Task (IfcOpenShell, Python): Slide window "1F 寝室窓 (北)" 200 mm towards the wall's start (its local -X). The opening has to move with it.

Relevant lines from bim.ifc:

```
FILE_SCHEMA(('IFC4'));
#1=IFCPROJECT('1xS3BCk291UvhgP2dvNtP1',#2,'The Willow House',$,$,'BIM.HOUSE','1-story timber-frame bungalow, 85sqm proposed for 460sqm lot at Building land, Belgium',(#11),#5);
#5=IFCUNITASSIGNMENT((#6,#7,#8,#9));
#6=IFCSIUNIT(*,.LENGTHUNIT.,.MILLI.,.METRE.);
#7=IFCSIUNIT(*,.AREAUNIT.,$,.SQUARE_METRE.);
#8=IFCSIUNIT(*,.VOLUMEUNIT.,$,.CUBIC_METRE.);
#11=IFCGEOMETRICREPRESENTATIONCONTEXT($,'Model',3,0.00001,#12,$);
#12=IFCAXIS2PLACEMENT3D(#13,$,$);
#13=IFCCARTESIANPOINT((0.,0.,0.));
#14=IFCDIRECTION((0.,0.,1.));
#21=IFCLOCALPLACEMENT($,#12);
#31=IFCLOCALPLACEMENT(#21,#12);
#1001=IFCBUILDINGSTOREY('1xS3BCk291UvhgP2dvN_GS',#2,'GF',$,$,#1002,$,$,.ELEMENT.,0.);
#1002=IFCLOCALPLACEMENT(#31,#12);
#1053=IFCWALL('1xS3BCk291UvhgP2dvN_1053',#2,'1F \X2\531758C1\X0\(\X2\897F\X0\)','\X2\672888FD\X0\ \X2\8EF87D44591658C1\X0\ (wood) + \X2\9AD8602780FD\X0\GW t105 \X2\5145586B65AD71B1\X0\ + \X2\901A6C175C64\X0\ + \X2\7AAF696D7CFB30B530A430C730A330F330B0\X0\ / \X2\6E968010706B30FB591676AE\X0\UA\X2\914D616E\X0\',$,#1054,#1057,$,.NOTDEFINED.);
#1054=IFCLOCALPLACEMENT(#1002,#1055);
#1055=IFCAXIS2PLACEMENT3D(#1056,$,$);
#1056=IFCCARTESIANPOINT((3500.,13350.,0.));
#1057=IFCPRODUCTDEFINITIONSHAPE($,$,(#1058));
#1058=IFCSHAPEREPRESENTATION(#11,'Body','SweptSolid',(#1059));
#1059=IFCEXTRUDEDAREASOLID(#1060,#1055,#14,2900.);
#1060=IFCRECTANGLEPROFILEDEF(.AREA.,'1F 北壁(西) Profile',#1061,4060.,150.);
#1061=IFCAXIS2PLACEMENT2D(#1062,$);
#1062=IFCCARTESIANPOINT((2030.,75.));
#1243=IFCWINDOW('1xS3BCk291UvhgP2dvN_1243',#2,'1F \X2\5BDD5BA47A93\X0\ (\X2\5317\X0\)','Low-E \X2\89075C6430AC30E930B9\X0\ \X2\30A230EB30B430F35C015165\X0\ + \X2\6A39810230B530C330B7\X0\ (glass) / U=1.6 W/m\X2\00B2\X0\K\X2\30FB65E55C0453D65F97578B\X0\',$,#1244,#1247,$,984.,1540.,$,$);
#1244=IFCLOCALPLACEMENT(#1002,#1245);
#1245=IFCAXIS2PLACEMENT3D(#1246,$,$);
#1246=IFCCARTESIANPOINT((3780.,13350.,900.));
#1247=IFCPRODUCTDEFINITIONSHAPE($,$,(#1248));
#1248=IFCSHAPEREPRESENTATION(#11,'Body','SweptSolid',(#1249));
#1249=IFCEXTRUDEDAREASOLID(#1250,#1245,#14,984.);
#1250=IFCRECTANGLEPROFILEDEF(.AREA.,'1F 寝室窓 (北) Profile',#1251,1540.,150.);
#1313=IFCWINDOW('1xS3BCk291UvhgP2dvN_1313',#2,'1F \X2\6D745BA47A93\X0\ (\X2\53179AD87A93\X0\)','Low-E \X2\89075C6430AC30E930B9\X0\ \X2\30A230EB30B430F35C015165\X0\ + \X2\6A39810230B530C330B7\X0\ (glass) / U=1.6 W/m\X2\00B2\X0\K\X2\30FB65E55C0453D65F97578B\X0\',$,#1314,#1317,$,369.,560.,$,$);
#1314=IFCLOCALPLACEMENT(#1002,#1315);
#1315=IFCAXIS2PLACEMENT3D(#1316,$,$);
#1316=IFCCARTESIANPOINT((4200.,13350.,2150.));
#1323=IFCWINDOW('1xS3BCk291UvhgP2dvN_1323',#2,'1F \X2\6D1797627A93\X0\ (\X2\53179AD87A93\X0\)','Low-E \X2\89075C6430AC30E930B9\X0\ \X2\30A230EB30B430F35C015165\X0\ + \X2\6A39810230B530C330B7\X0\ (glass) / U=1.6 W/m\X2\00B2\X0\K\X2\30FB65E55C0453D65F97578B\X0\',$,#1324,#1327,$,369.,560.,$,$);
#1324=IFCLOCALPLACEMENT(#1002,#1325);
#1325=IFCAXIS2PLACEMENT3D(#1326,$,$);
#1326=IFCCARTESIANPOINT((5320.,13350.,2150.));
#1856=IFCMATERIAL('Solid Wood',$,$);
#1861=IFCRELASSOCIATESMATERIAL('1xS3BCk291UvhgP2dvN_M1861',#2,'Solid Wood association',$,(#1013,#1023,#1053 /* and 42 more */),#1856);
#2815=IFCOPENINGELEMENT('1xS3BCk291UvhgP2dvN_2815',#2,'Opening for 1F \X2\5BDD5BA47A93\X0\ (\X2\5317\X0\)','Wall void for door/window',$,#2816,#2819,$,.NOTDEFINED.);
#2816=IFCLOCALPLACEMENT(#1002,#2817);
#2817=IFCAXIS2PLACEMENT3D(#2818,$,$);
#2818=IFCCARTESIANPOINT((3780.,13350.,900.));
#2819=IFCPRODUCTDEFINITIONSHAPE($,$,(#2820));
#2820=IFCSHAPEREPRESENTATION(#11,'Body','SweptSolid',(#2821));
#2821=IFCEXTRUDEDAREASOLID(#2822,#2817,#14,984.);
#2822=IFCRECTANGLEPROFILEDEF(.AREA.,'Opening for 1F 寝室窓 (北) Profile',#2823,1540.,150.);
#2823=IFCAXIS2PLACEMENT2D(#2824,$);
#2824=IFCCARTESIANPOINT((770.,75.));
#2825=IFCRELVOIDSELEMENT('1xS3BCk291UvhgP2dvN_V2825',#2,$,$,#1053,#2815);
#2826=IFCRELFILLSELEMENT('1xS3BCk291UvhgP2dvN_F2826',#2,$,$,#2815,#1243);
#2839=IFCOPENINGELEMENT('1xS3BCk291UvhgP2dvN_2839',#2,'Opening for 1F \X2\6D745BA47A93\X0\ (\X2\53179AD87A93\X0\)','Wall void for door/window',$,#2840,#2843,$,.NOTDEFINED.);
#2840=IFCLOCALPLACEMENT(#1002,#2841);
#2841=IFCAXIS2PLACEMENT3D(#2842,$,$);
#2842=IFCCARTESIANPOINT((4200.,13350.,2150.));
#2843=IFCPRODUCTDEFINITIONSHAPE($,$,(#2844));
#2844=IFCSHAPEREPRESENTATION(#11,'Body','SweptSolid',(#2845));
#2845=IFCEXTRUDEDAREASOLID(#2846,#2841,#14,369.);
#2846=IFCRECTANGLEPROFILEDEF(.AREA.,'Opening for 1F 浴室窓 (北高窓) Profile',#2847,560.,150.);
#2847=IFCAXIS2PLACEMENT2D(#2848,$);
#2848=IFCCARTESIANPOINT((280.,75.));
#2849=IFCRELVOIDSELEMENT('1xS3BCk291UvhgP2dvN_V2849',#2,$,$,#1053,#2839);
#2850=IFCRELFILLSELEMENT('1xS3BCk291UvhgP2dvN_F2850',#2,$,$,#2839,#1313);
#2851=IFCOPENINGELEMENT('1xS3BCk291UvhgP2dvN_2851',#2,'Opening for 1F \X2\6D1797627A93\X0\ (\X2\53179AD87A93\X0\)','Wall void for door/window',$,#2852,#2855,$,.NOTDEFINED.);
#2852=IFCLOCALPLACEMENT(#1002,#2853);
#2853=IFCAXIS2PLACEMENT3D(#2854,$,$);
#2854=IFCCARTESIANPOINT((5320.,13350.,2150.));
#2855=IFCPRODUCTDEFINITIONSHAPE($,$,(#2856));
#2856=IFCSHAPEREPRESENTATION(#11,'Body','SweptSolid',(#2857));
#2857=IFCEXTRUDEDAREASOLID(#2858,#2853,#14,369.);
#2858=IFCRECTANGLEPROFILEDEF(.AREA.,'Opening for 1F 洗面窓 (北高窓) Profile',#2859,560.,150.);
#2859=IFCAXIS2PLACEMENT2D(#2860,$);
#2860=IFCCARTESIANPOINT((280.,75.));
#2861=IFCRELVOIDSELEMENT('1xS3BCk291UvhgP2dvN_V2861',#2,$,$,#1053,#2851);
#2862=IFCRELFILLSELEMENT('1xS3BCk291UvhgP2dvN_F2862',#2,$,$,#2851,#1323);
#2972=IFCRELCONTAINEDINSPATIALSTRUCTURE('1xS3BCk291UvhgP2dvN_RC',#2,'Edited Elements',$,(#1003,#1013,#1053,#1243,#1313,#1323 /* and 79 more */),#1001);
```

```python
import ifcopenshell
import ifcopenshell.api.geometry
import ifcopenshell.util.placement
import ifcopenshell.util.unit

model = ifcopenshell.open("bim.ifc")
unit_scale = ifcopenshell.util.unit.calculate_unit_scale(model)

window = model.by_id(1243)
opening = window.FillsVoids[0].RelatingOpeningElement
wall = opening.VoidsElements[0].RelatingBuildingElement

wall_matrix = ifcopenshell.util.placement.get_local_placement(wall.ObjectPlacement)
shift = wall_matrix[:3, 0] * -0.2 / unit_scale
before = ifcopenshell.util.placement.get_local_placement(window.ObjectPlacement)[:3, 3].copy()

# The window is not placed relative to its opening, so move both.
for product in (opening, window):
    matrix = ifcopenshell.util.placement.get_local_placement(product.ObjectPlacement)
    matrix[:3, 3] += shift
    ifcopenshell.api.geometry.edit_object_placement(model, product=product, matrix=matrix, is_si=False)

after = ifcopenshell.util.placement.get_local_placement(window.ObjectPlacement)[:3, 3]
print("window moved by", (after - before).round(3) + 0.0)

model.write("bim-out.ifc")
```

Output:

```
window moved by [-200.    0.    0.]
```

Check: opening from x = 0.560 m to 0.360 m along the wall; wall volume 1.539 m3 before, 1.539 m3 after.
